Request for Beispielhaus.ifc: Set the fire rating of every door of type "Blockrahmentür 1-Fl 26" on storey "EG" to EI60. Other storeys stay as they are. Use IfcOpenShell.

First a look at what the model holds.

```python
import ifcopenshell
import ifcopenshell.util.element

model = ifcopenshell.open("Beispielhaus.ifc")
print(model.schema)
storey = next(s for s in model.by_type("IfcBuildingStorey") if s.Name == "EG")
doors = [e for e in ifcopenshell.util.element.get_decomposition(storey) if e.is_a("IfcDoor")]
seen = {}
for e in doors:
    element_type = ifcopenshell.util.element.get_type(e)
    key = (element_type.Name if element_type != e and element_type else None, ifcopenshell.util.element.get_pset(e, "Pset_DoorCommon", "FireRating"))
    seen[key] = seen.get(key, 0) + 1
for (name, value), count in sorted(seen.items(), key=str):
    print(count, "x", name, "|", value)
```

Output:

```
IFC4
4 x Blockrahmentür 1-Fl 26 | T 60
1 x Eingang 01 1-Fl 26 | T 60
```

```python
import ifcopenshell
import ifcopenshell.api.pset
import ifcopenshell.util.element

model = ifcopenshell.open("Beispielhaus.ifc")

storey = next(s for s in model.by_type("IfcBuildingStorey") if s.Name == "EG")
doors = [e for e in ifcopenshell.util.element.get_decomposition(storey) if e.is_a("IfcDoor")]

count = 0
for e in doors:
    element_type = ifcopenshell.util.element.get_type(e)
    if element_type in (None, e) or element_type.Name != "Blockrahmentür 1-Fl 26":
        continue
    # add_pset returns the element's existing set when there is one.
    pset = ifcopenshell.api.pset.add_pset(model, product=e, name="Pset_DoorCommon")
    ifcopenshell.api.pset.edit_pset(model, pset=pset, properties={"FireRating": "EI60"})
    count += 1

print(count, "doors updated")

model.write("Beispielhaus-out.ifc")
```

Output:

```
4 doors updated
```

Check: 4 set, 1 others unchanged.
